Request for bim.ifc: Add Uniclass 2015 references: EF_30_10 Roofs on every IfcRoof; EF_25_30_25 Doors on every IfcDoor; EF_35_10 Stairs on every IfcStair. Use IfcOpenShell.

First a look at what the model holds.

```python
import ifcopenshell

model = ifcopenshell.open("bim.ifc")
print(model.schema)
print("classifications:", [c.Name for c in model.by_type("IfcClassification")])
for ifc_class in ("IfcDoor", "IfcRoof", "IfcStair", "IfcWall", "IfcWindow"):
    print(ifc_class, len(model.by_type(ifc_class)))
```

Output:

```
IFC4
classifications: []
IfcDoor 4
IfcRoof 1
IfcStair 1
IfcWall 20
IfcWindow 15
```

```python
import ifcopenshell
import ifcopenshell.api.classification

model = ifcopenshell.open("bim.ifc")

system = ifcopenshell.api.classification.add_classification(model, classification="Uniclass 2015")

codes = {
    "IfcRoof": ("EF_30_10", "Roofs"),
    "IfcDoor": ("EF_25_30_25", "Doors"),
    "IfcStair": ("EF_35_10", "Stairs"),
}
for ifc_class, (code, name) in codes.items():
    products = model.by_type(ifc_class)
    ifcopenshell.api.classification.add_reference(
        model, products=products, classification=system, identification=code, name=name
    )
    print(code, len(products))

model.write("bim_rev.ifc")
```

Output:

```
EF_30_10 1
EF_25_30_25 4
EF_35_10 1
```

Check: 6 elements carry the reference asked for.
